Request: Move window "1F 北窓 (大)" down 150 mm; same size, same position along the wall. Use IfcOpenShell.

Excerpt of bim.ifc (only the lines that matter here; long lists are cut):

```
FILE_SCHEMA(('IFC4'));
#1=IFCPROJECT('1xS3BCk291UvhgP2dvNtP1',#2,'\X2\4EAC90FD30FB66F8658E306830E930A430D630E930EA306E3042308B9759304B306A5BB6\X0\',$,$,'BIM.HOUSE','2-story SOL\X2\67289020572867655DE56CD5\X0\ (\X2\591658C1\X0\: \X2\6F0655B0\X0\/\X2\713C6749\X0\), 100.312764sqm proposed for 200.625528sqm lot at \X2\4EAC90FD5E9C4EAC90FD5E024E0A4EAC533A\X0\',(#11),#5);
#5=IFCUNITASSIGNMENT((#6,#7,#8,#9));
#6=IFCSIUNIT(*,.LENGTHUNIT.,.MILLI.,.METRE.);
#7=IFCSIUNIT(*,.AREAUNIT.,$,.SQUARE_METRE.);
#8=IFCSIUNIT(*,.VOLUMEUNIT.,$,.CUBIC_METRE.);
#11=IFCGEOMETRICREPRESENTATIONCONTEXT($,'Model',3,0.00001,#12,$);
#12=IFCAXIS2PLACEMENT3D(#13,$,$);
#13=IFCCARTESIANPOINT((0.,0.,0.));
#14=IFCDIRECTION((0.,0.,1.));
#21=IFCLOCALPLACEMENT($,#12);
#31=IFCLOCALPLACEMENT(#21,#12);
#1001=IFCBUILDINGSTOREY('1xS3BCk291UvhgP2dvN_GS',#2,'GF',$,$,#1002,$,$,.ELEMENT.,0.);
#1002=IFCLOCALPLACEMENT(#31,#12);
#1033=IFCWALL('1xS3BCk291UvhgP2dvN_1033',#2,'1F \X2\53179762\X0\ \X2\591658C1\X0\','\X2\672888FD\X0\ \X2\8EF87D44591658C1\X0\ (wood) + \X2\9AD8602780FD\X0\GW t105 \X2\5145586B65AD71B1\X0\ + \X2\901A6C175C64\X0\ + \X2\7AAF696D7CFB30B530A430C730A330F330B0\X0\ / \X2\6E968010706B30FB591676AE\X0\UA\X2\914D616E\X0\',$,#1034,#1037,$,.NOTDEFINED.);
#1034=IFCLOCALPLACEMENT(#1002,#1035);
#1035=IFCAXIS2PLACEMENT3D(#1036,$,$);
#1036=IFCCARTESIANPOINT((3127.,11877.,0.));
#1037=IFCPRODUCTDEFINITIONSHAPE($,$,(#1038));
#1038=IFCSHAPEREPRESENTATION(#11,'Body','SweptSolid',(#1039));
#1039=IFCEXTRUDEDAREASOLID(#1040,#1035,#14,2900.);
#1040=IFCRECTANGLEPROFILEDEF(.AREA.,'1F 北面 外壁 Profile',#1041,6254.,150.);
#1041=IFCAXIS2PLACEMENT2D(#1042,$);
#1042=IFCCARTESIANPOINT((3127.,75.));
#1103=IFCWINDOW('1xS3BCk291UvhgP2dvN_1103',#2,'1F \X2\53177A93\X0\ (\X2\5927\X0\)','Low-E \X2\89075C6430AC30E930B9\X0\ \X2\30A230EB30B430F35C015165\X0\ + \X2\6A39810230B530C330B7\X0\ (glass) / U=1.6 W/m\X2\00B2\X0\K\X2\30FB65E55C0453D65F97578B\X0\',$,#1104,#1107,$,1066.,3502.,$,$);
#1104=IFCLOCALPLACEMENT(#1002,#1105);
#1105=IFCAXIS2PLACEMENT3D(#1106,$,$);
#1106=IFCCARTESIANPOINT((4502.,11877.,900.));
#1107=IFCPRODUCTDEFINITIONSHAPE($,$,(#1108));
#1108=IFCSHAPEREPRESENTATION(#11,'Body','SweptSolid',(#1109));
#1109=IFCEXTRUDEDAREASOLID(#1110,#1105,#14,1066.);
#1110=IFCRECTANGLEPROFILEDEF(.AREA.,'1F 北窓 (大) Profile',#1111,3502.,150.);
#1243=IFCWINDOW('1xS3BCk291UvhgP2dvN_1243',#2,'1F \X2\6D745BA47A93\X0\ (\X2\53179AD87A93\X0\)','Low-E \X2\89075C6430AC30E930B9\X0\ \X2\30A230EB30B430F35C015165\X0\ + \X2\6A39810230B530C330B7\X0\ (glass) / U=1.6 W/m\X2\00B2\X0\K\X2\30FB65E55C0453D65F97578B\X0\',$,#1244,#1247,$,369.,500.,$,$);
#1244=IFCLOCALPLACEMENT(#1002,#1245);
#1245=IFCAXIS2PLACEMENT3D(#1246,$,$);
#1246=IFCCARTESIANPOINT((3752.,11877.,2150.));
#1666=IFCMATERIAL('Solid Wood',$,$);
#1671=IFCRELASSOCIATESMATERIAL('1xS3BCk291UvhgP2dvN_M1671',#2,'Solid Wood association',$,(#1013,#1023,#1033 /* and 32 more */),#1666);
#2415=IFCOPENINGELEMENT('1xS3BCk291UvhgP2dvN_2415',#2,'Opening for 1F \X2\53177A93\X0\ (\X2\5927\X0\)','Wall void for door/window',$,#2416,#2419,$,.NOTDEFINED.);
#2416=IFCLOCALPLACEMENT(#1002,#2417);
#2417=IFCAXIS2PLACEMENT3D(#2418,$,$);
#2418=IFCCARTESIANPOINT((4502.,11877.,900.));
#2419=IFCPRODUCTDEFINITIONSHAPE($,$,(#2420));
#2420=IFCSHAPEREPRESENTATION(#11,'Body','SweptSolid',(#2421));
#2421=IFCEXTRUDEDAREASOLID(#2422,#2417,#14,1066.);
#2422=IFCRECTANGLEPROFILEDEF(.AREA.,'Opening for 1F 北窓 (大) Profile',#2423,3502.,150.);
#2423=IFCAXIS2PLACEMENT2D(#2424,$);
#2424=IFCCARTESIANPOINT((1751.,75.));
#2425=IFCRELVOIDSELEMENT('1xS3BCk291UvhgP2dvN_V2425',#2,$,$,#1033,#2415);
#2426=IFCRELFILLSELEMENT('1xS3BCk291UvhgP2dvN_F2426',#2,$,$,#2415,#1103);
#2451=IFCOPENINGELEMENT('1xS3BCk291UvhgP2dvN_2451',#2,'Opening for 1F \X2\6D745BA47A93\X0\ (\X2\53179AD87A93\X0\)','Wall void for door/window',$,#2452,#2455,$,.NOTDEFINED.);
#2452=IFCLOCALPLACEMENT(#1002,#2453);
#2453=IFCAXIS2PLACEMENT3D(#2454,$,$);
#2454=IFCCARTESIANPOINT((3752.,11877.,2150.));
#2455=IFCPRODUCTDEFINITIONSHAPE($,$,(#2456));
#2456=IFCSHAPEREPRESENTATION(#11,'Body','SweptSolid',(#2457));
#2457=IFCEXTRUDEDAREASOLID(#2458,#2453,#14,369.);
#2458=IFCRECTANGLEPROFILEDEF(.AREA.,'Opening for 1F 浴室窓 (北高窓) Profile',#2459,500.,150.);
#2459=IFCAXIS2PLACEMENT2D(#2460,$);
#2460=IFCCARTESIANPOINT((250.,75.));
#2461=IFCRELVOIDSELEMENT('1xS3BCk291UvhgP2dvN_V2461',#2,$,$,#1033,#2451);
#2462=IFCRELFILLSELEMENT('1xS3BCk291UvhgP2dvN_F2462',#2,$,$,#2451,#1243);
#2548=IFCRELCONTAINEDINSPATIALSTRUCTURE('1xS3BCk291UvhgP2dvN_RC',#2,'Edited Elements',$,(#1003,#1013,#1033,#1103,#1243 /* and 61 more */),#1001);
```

```python
import numpy as np
import ifcopenshell
import ifcopenshell.api.geometry
import ifcopenshell.util.placement
import ifcopenshell.util.unit

model = ifcopenshell.open("bim.ifc")
unit_scale = ifcopenshell.util.unit.calculate_unit_scale(model)

window = model.by_id(1103)
opening = window.FillsVoids[0].RelatingOpeningElement
dz = -150.0

shift = np.array([0.0, 0.0, dz])
# The window is not placed relative to its opening, so move both.
for product in (opening, window):
    matrix = ifcopenshell.util.placement.get_local_placement(product.ObjectPlacement)
    matrix[:3, 3] += shift
    ifcopenshell.api.geometry.edit_object_placement(model, product=product, matrix=matrix, is_si=False)

print(f"moved by {dz * unit_scale:+.3f} m")

model.write("bim-out.ifc")
```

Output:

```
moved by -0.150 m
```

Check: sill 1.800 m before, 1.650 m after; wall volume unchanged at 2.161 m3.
